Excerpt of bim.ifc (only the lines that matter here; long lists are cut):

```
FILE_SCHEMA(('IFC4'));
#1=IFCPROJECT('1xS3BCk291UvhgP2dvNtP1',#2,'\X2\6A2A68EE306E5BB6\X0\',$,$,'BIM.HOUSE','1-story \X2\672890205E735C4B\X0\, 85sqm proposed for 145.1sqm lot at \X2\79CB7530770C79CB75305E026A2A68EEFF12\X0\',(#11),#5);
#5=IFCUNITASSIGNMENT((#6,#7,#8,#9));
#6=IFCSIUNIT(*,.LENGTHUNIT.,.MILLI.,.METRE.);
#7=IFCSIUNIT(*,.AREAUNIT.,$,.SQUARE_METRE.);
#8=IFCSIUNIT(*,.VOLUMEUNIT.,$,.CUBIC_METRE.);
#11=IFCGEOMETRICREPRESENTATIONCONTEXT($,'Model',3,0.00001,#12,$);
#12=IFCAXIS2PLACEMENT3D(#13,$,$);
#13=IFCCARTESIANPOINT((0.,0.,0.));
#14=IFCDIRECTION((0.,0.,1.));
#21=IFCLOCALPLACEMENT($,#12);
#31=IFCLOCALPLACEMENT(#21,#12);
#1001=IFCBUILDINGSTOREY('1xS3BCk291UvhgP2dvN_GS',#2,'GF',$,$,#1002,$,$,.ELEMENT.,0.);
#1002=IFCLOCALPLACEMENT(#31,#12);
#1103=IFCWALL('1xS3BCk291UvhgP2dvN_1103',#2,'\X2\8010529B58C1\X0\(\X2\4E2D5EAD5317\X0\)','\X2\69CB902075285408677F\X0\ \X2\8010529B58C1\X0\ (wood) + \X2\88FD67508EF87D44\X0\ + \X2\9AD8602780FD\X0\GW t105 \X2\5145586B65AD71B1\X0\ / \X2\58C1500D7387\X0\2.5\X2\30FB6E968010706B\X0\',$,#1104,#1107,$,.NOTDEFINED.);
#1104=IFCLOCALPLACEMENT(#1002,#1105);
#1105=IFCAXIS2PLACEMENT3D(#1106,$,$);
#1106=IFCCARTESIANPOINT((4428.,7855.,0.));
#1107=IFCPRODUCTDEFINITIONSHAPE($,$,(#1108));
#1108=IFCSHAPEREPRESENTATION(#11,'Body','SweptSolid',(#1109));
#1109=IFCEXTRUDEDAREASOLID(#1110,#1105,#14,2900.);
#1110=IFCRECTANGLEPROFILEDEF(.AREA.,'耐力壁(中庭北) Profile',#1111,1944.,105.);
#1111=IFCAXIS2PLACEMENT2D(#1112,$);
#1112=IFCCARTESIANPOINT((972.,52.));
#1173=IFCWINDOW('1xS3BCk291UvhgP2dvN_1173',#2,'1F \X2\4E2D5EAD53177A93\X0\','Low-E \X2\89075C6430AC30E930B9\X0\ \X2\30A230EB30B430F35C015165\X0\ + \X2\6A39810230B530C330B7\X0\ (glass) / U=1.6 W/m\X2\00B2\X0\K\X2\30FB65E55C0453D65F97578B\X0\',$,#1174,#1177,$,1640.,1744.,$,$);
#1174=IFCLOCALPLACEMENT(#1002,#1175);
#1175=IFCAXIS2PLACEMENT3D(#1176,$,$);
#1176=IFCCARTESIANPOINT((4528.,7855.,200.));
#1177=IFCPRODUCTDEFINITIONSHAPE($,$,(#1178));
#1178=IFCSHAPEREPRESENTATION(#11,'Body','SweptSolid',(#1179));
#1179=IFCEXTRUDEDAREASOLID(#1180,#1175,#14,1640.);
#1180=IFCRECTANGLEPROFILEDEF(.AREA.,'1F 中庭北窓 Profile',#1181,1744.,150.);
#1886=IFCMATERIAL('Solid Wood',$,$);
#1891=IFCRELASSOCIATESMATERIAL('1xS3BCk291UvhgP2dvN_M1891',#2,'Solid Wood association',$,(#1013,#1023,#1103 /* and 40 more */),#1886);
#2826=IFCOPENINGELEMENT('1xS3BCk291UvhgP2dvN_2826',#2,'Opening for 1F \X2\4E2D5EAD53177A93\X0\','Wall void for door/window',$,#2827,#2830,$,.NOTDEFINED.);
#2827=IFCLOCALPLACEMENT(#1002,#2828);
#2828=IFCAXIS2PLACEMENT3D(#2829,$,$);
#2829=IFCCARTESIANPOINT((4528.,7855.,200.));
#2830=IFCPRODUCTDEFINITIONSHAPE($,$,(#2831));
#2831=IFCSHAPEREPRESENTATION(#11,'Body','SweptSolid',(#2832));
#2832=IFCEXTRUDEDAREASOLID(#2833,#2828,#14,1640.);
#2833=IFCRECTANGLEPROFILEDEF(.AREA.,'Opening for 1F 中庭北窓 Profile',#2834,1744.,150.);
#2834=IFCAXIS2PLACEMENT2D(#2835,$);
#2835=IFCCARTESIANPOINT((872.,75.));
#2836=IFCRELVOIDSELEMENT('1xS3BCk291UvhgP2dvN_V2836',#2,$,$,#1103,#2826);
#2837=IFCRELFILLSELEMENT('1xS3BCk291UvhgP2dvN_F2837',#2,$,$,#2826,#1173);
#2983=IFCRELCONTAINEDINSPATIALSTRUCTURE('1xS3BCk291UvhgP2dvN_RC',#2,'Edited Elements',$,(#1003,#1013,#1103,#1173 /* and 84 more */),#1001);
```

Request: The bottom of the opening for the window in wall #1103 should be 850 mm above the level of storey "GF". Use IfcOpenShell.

```python
import numpy as np
import ifcopenshell
import ifcopenshell.api.geometry
import ifcopenshell.geom
import ifcopenshell.util.element
import ifcopenshell.util.placement
import ifcopenshell.util.shape
import ifcopenshell.util.unit

model = ifcopenshell.open("bim.ifc")
unit_scale = ifcopenshell.util.unit.calculate_unit_scale(model)

window = model.by_guid("1xS3BCk291UvhgP2dvN_1173")
opening = window.FillsVoids[0].RelatingOpeningElement
storey = ifcopenshell.util.element.get_container(window, ifc_class="IfcBuildingStorey")
level = ifcopenshell.util.placement.get_local_placement(storey.ObjectPlacement)[2, 3]

# The opening's origin need not be at the sill, so measure its lowest point.
shape = ifcopenshell.geom.create_shape(ifcopenshell.geom.settings(), opening)
bottom = ifcopenshell.util.shape.get_shape_bottom_elevation(shape, shape.geometry) / unit_scale
dz = level + 0.85 / unit_scale - bottom

shift = np.array([0.0, 0.0, dz])
# The window is not placed relative to its opening, so move both.
for product in (opening, window):
    matrix = ifcopenshell.util.placement.get_local_placement(product.ObjectPlacement)
    matrix[:3, 3] += shift
    ifcopenshell.api.geometry.edit_object_placement(model, product=product, matrix=matrix, is_si=False)

print(f"moved by {dz * unit_scale:+.3f} m")

model.write("bim_rev.ifc")
```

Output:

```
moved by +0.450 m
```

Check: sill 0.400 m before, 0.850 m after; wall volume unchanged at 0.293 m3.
